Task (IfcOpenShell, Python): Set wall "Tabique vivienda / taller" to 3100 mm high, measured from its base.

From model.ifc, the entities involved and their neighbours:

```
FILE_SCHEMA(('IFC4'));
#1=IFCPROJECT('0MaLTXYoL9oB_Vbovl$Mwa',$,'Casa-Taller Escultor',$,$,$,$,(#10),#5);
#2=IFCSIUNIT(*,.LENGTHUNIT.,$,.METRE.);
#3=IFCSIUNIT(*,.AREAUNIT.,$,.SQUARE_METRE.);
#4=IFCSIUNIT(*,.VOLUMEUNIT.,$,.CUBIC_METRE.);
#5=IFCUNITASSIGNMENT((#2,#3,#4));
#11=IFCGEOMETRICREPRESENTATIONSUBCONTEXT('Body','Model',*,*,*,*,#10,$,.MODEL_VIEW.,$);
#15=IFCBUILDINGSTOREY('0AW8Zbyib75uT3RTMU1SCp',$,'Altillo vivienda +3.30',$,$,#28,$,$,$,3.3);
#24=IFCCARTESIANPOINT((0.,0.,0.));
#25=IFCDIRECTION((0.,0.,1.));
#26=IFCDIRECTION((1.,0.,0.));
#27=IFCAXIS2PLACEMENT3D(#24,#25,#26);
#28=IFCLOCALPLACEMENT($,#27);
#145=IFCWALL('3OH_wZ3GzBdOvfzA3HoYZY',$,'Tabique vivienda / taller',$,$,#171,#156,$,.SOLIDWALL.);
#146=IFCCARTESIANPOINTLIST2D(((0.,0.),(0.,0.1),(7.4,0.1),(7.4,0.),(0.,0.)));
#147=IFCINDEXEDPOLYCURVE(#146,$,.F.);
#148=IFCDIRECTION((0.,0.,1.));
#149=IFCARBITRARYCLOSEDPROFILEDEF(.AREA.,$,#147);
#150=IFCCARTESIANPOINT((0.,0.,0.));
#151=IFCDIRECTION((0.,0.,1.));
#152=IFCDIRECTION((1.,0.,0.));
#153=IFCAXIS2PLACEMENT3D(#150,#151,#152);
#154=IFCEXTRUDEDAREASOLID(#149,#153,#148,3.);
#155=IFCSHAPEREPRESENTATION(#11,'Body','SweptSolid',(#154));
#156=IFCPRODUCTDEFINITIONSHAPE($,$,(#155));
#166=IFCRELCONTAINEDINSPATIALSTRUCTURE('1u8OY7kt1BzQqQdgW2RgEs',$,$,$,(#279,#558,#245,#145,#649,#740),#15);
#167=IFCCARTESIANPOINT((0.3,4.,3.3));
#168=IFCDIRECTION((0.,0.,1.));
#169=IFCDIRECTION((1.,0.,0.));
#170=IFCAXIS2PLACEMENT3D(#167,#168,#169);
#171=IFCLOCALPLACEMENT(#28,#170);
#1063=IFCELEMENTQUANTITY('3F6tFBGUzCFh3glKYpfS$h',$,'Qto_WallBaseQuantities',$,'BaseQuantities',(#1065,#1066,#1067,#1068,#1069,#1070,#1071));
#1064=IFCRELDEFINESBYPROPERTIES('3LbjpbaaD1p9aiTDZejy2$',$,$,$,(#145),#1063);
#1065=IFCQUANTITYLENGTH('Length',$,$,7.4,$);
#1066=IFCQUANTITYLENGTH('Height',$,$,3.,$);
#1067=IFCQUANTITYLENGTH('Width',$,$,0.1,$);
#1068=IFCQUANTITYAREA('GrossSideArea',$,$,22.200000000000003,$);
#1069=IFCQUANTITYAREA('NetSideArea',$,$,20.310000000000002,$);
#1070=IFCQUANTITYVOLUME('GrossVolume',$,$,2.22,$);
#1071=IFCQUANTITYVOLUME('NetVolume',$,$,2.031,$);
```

```python
import ifcopenshell
import ifcopenshell.api.pset
import ifcopenshell.geom
import ifcopenshell.util.element
import ifcopenshell.util.representation
import ifcopenshell.util.shape
import ifcopenshell.util.unit

model = ifcopenshell.open("model.ifc")
unit_scale = ifcopenshell.util.unit.calculate_unit_scale(model)
area_scale = ifcopenshell.util.unit.calculate_unit_scale(model, "AREAUNIT")
volume_scale = ifcopenshell.util.unit.calculate_unit_scale(model, "VOLUMEUNIT")
settings = ifcopenshell.geom.settings()


def volume(element):
    """Net volume in cubic metres, openings subtracted."""
    shape = ifcopenshell.geom.create_shape(settings, element)
    return ifcopenshell.util.shape.get_volume(shape.geometry)


wall = model.by_guid("3OH_wZ3GzBdOvfzA3HoYZY")
before = volume(wall)

body = ifcopenshell.util.representation.get_representation(wall, "Model", "Body")
solid = body.Items[0]
old_height = solid.Depth
solid.Depth = 3.1 / unit_scale
after = volume(wall)
thickness = 0.1  # wall thickness in metres

# Update the stored height, areas and volumes.
qto = model.by_id(ifcopenshell.util.element.get_pset(wall, "Qto_WallBaseQuantities", should_inherit=False)["id"])
ifcopenshell.api.pset.edit_qto(model, qto=qto, properties={
    "Height": solid.Depth,
    "GrossSideArea": ifcopenshell.util.element.get_pset(wall, "Qto_WallBaseQuantities", "GrossSideArea") * solid.Depth / old_height,
    "NetSideArea": after / thickness / area_scale,
    "GrossVolume": ifcopenshell.util.element.get_pset(wall, "Qto_WallBaseQuantities", "GrossVolume") * solid.Depth / old_height,
    "NetVolume": after / volume_scale,
})

print(f"height {old_height:g} -> {solid.Depth:g}, volume {before:.3f} -> {after:.3f} m3")

model.write("model_rev.ifc")
```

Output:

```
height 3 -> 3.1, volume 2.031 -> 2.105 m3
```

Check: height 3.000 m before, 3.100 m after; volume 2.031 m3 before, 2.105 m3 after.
